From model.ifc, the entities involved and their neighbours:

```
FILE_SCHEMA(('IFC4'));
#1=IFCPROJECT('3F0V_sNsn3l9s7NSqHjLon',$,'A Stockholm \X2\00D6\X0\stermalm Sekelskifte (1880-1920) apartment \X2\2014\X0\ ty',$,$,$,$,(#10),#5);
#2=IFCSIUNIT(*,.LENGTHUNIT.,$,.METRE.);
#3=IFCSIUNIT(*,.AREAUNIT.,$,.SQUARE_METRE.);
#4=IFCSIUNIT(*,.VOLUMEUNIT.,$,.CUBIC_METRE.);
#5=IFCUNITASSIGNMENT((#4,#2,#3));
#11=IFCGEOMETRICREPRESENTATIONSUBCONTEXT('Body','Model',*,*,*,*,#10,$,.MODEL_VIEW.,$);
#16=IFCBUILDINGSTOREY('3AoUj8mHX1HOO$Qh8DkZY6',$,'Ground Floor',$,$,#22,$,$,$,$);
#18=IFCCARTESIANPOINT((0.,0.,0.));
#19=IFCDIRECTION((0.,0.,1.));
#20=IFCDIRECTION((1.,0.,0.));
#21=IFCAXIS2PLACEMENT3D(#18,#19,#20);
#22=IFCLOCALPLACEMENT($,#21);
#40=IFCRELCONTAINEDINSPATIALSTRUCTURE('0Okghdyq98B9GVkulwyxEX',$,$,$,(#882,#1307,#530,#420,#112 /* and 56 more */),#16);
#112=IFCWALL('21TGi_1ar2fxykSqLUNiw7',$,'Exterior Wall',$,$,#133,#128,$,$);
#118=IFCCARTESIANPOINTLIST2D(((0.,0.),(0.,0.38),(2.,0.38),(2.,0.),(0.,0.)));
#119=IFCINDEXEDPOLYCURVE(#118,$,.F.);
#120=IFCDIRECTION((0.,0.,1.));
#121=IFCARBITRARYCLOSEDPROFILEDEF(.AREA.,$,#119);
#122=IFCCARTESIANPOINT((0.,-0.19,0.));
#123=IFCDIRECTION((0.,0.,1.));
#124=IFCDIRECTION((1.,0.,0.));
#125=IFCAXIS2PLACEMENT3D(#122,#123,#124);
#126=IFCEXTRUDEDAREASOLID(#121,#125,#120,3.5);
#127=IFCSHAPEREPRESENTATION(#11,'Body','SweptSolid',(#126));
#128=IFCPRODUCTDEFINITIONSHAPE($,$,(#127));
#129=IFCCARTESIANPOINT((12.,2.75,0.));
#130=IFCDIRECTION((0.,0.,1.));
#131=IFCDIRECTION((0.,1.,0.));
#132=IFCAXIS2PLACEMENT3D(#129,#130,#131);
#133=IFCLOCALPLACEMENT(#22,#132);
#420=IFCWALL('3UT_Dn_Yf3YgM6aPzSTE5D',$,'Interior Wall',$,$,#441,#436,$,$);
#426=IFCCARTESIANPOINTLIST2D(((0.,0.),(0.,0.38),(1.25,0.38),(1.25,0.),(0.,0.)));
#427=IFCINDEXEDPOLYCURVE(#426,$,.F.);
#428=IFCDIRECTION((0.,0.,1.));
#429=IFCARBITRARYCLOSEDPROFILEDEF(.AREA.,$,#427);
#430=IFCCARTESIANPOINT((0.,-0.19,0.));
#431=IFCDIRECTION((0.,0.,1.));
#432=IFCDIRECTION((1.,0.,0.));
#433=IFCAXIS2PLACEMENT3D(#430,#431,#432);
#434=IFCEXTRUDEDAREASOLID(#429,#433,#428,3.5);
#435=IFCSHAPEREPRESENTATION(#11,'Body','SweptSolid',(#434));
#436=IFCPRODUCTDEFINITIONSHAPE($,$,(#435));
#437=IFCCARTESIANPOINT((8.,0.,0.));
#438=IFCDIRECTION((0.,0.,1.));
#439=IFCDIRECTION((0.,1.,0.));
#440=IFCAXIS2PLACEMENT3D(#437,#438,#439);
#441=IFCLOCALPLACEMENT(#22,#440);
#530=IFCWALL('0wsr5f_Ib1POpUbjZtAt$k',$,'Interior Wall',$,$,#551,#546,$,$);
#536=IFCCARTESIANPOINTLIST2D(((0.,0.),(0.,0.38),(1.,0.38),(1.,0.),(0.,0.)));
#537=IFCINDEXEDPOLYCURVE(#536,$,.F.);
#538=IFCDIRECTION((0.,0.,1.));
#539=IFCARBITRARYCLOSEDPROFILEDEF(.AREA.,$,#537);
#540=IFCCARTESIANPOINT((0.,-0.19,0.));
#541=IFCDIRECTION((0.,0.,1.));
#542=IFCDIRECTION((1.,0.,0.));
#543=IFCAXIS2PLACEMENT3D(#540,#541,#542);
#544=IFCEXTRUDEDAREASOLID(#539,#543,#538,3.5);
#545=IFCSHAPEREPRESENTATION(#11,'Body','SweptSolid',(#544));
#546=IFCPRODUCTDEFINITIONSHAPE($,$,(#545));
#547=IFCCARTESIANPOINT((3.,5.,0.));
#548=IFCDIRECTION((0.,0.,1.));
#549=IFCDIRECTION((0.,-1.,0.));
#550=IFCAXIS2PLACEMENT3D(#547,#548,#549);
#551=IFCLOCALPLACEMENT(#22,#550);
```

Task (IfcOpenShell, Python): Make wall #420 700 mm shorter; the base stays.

```python
import ifcopenshell
import ifcopenshell.geom
import ifcopenshell.util.representation
import ifcopenshell.util.shape
import ifcopenshell.util.unit

model = ifcopenshell.open("model.ifc")
unit_scale = ifcopenshell.util.unit.calculate_unit_scale(model)
settings = ifcopenshell.geom.settings()


def volume(element):
    """Net volume in cubic metres, openings subtracted."""
    shape = ifcopenshell.geom.create_shape(settings, element)
    return ifcopenshell.util.shape.get_volume(shape.geometry)


wall = model.by_id(420)
before = volume(wall)

body = ifcopenshell.util.representation.get_representation(wall, "Model", "Body")
solid = body.Items[0]
old_height = solid.Depth
solid.Depth -= 0.7 / unit_scale
after = volume(wall)

print(f"height {old_height:g} -> {solid.Depth:g}, volume {before:.3f} -> {after:.3f} m3")

model.write("model-out.ifc")
```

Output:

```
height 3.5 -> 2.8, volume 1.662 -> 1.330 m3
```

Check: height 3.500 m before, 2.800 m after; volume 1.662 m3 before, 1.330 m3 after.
